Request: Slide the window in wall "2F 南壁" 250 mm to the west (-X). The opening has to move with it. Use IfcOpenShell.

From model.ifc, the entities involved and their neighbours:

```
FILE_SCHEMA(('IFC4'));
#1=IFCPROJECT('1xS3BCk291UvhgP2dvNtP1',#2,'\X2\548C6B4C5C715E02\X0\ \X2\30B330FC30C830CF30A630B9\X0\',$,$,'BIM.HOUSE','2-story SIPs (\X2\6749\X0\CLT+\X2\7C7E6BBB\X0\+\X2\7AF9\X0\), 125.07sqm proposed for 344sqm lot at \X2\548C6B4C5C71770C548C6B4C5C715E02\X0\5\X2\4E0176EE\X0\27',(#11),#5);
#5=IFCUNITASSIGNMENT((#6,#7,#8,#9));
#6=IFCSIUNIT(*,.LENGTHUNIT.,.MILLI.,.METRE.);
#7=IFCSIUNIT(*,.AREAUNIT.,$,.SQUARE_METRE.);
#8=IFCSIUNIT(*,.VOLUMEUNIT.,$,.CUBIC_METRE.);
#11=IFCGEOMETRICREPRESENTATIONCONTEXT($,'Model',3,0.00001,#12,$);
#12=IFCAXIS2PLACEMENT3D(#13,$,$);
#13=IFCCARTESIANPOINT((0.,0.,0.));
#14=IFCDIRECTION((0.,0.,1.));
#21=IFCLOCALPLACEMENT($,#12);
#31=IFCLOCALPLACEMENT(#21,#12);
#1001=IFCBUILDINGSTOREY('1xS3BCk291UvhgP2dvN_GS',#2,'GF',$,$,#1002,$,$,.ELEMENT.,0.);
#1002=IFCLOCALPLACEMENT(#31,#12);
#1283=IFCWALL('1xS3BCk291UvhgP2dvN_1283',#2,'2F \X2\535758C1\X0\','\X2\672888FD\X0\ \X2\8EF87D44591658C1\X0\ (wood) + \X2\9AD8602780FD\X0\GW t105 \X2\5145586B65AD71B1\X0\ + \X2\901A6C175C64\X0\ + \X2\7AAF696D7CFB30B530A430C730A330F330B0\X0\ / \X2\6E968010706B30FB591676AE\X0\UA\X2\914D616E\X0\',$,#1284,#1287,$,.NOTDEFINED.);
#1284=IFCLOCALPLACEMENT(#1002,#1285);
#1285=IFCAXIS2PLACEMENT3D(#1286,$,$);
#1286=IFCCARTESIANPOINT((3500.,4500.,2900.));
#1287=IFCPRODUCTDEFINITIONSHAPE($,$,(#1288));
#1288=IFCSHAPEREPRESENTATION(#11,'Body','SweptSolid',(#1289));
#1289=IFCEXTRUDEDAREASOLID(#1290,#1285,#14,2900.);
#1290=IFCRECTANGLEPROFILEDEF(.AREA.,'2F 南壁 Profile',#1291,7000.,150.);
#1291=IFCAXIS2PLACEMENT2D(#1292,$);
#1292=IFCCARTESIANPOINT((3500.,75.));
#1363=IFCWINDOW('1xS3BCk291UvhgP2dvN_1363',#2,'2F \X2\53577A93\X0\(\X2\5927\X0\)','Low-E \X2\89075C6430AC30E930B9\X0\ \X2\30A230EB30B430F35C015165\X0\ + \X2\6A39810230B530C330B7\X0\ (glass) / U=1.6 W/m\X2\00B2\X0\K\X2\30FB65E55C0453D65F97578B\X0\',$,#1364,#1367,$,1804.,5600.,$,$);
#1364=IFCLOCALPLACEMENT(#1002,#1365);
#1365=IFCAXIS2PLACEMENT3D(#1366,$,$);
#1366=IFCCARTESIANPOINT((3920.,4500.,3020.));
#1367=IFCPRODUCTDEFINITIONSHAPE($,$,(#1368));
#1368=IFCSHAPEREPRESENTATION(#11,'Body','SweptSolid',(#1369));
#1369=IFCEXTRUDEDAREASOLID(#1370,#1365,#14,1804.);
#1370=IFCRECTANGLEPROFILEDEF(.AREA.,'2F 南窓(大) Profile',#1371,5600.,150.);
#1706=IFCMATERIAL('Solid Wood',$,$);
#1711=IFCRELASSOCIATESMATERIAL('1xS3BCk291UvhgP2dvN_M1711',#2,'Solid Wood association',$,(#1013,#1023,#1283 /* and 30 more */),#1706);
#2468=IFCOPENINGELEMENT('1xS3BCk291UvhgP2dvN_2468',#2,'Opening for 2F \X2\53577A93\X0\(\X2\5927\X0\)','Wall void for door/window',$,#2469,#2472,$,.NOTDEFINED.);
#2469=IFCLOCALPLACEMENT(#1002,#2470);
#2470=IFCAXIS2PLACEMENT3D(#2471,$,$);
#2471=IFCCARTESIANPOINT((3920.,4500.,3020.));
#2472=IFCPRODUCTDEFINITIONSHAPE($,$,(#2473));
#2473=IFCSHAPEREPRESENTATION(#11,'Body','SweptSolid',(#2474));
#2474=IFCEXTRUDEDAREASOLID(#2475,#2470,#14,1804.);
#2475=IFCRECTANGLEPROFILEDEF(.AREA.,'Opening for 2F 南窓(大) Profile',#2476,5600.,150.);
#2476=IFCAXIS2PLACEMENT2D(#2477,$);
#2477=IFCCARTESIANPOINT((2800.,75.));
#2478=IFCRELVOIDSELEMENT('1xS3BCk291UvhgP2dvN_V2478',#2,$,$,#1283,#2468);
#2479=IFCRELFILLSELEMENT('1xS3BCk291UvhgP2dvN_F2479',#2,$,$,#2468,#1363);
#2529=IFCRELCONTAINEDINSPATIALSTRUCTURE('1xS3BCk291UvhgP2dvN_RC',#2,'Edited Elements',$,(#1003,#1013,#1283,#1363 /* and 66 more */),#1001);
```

```python
import ifcopenshell
import ifcopenshell.api.geometry
import ifcopenshell.util.placement
import ifcopenshell.util.unit

model = ifcopenshell.open("model.ifc")
unit_scale = ifcopenshell.util.unit.calculate_unit_scale(model)

window = model.by_guid("1xS3BCk291UvhgP2dvN_1363")
opening = window.FillsVoids[0].RelatingOpeningElement
wall = opening.VoidsElements[0].RelatingBuildingElement

wall_matrix = ifcopenshell.util.placement.get_local_placement(wall.ObjectPlacement)
shift = wall_matrix[:3, 0] * -0.25 / unit_scale
before = ifcopenshell.util.placement.get_local_placement(window.ObjectPlacement)[:3, 3].copy()

# The window is not placed relative to its opening, so move both.
for product in (opening, window):
    matrix = ifcopenshell.util.placement.get_local_placement(product.ObjectPlacement)
    matrix[:3, 3] += shift
    ifcopenshell.api.geometry.edit_object_placement(model, product=product, matrix=matrix, is_si=False)

after = ifcopenshell.util.placement.get_local_placement(window.ObjectPlacement)[:3, 3]
print("window moved by", (after - before).round(3) + 0.0)

model.write("model_edited.ifc")
```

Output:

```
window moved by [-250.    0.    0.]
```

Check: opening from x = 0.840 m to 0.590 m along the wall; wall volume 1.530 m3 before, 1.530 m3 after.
